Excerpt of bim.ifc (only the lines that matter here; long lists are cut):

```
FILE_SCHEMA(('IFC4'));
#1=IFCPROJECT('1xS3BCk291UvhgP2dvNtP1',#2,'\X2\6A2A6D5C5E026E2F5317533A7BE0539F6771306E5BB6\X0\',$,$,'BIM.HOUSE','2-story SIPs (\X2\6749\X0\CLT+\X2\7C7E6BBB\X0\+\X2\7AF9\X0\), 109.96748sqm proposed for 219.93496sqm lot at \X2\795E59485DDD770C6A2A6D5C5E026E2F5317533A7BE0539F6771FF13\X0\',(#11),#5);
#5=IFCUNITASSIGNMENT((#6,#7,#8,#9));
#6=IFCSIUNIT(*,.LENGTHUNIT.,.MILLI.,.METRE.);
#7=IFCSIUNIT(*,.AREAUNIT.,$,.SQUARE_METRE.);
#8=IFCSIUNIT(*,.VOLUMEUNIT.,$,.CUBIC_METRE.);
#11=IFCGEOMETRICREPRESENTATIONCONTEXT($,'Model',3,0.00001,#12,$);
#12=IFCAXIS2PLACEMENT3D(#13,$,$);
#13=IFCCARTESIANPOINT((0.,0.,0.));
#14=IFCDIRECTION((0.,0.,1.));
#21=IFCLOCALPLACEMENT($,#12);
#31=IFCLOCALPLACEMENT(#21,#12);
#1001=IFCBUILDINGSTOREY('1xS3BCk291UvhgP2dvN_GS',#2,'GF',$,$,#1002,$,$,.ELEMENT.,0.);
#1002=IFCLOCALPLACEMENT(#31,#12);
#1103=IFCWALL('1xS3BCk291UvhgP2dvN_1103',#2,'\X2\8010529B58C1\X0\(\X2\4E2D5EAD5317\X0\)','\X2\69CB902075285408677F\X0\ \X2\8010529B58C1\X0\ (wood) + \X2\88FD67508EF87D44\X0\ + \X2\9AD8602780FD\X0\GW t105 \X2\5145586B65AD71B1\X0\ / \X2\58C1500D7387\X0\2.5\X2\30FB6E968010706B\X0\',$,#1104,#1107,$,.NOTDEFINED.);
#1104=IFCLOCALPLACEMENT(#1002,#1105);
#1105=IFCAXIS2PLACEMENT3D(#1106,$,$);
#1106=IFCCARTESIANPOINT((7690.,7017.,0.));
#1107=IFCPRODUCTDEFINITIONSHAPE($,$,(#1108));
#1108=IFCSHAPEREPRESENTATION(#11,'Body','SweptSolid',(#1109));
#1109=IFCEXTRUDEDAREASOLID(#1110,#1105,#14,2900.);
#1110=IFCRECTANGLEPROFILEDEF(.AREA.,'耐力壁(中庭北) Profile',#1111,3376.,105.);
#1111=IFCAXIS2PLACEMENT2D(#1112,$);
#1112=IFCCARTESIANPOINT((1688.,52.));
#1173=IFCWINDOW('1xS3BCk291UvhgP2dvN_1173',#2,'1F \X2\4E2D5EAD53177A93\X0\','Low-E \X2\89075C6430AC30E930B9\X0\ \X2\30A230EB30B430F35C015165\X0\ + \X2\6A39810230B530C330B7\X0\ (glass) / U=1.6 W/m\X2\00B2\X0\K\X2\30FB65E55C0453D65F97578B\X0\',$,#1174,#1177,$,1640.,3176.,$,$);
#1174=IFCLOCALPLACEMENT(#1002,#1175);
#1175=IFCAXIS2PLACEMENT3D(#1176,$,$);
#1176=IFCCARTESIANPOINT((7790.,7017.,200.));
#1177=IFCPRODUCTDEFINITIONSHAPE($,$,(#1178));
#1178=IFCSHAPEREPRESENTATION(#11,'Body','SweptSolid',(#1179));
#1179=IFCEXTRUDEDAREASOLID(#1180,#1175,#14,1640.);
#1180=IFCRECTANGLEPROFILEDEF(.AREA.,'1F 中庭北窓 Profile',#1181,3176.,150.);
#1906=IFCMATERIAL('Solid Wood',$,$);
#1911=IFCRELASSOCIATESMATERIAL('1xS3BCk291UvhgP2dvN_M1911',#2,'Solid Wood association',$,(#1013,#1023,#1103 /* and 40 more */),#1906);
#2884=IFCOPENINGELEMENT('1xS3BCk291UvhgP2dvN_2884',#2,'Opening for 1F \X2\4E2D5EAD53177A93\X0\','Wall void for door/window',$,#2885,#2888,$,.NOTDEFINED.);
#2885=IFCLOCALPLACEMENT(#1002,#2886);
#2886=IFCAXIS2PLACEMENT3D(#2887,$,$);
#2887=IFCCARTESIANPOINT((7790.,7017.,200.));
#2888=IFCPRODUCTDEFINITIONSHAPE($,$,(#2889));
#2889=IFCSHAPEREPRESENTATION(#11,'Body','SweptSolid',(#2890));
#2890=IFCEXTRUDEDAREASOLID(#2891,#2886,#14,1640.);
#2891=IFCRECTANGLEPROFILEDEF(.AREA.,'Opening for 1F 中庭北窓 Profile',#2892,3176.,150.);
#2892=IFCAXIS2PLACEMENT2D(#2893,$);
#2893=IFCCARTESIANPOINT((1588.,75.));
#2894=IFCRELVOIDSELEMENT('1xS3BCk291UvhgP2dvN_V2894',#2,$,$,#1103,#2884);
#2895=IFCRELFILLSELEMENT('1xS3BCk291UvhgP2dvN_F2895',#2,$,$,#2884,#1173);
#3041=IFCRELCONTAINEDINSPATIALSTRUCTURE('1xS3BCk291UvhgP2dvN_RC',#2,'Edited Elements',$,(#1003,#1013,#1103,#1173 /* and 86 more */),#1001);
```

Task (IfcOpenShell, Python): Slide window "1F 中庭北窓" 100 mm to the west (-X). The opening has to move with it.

```python
import ifcopenshell
import ifcopenshell.api.geometry
import ifcopenshell.util.placement
import ifcopenshell.util.unit

model = ifcopenshell.open("bim.ifc")
unit_scale = ifcopenshell.util.unit.calculate_unit_scale(model)

window = model.by_guid("1xS3BCk291UvhgP2dvN_1173")
opening = window.FillsVoids[0].RelatingOpeningElement
wall = opening.VoidsElements[0].RelatingBuildingElement

wall_matrix = ifcopenshell.util.placement.get_local_placement(wall.ObjectPlacement)
shift = wall_matrix[:3, 0] * -0.1 / unit_scale
before = ifcopenshell.util.placement.get_local_placement(window.ObjectPlacement)[:3, 3].copy()

# The window is not placed relative to its opening, so move both.
for product in (opening, window):
    matrix = ifcopenshell.util.placement.get_local_placement(product.ObjectPlacement)
    matrix[:3, 3] += shift
    ifcopenshell.api.geometry.edit_object_placement(model, product=product, matrix=matrix, is_si=False)

after = ifcopenshell.util.placement.get_local_placement(window.ObjectPlacement)[:3, 3]
print("window moved by", (after - before).round(3) + 0.0)

model.write("bim_v2.ifc")
```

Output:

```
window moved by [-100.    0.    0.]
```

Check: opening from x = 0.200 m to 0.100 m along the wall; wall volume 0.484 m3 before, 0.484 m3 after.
